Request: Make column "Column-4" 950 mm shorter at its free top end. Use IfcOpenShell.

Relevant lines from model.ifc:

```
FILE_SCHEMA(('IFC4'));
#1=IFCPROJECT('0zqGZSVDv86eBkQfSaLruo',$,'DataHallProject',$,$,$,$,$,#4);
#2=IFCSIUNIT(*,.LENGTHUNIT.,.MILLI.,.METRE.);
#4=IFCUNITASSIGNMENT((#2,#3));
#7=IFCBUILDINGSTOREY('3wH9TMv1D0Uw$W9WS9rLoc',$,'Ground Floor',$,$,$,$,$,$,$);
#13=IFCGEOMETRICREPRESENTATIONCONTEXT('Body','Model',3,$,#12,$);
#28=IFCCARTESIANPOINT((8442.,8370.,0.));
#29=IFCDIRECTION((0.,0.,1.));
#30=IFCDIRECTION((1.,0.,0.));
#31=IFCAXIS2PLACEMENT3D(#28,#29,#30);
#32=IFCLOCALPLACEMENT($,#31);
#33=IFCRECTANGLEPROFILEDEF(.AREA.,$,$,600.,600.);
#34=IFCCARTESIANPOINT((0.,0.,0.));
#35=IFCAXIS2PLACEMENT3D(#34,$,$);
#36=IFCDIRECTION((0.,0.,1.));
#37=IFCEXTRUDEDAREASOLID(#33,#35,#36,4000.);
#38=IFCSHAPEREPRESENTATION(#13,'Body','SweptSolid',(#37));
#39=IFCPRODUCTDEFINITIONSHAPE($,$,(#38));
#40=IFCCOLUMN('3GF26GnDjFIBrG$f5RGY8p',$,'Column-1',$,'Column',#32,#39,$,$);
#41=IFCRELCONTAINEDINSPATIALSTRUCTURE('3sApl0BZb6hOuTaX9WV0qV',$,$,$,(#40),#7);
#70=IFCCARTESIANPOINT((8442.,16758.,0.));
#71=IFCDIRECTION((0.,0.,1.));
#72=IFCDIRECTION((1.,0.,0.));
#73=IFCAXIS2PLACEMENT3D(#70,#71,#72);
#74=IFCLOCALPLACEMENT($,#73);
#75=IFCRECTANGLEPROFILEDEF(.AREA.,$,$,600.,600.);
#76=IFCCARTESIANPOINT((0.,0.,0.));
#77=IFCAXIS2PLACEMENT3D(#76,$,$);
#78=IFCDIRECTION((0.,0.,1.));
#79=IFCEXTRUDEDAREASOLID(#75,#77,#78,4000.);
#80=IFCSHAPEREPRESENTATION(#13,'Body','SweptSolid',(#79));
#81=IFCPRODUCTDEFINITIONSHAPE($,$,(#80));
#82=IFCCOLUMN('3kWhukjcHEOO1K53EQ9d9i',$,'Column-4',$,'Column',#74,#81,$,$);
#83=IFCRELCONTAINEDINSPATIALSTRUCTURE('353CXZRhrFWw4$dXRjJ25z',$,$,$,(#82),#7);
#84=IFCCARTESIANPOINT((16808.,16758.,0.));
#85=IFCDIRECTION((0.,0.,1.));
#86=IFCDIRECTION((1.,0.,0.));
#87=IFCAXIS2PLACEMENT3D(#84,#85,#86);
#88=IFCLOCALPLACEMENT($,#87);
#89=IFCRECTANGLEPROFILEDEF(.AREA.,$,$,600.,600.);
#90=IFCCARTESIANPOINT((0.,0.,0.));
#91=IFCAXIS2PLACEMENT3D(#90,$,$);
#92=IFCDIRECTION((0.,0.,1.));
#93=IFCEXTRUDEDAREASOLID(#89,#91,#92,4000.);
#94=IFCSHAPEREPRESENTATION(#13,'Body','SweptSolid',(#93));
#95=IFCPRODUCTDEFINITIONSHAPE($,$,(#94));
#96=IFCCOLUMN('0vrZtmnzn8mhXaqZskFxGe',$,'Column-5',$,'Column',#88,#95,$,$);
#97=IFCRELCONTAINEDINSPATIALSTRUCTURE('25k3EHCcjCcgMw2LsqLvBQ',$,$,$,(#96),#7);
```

```python
import ifcopenshell

model = ifcopenshell.open("model.ifc")

member = model.by_guid("3kWhukjcHEOO1K53EQ9d9i")
change = -950.0

# The extrusion runs towards the end named, so only its depth changes.
body = next(r for r in member.Representation.Representations if r.RepresentationIdentifier == "Body")
solid = body.Items[0]
old_length = solid.Depth
solid.Depth += change

print(f"length {old_length:g} -> {solid.Depth:g}")

model.write("model-out.ifc")
```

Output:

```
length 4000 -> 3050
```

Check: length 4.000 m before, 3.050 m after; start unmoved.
